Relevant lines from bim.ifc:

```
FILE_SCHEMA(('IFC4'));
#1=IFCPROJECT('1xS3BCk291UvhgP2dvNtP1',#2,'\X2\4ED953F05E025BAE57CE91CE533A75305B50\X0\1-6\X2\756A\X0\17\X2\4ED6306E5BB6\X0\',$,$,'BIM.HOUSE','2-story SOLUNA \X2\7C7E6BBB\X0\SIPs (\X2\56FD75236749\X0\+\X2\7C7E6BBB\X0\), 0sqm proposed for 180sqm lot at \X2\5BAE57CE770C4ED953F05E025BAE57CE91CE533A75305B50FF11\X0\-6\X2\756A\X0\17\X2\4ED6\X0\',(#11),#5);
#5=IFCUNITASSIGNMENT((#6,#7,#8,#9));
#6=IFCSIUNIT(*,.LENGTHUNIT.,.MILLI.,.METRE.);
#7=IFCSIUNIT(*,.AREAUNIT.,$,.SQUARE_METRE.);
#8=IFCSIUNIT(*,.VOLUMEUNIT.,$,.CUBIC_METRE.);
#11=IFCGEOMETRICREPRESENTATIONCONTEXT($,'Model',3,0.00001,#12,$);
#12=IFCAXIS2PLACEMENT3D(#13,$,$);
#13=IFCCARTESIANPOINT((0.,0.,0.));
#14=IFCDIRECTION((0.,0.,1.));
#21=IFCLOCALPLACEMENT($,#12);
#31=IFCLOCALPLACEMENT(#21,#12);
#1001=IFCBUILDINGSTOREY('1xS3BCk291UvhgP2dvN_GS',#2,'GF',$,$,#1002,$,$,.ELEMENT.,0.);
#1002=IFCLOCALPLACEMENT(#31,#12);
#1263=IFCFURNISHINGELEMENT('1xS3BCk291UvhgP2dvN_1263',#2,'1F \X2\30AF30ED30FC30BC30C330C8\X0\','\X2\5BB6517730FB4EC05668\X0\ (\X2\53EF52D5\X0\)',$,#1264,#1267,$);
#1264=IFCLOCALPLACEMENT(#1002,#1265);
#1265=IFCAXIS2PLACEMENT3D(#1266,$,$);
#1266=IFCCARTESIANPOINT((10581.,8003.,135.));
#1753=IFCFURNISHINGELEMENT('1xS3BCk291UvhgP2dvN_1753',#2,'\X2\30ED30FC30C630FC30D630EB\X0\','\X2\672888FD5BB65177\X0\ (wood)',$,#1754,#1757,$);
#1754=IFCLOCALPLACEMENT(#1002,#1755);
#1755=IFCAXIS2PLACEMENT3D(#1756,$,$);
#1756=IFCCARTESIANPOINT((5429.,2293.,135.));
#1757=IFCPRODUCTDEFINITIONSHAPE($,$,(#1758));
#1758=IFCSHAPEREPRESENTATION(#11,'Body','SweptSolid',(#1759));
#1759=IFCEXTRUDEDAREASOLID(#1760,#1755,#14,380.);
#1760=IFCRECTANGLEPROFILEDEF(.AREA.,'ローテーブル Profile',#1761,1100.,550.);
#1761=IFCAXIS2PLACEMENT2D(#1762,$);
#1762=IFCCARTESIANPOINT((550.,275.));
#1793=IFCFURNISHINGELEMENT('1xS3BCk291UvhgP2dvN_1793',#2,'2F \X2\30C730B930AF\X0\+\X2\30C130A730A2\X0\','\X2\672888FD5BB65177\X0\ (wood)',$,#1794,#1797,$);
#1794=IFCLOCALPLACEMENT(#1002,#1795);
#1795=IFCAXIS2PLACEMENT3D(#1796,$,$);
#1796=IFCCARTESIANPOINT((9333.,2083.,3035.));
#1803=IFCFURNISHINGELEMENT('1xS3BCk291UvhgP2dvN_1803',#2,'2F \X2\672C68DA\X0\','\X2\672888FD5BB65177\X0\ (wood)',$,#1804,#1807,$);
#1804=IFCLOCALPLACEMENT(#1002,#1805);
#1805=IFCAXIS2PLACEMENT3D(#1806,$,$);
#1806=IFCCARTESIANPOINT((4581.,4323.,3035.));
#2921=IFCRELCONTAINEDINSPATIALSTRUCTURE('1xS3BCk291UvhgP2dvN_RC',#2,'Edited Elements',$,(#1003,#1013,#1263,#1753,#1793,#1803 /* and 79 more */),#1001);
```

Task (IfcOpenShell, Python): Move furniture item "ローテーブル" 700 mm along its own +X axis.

```python
import ifcopenshell
import ifcopenshell.api.geometry
import ifcopenshell.util.placement
import ifcopenshell.util.unit

model = ifcopenshell.open("bim.ifc")
unit_scale = ifcopenshell.util.unit.calculate_unit_scale(model)

item = model.by_guid("1xS3BCk291UvhgP2dvN_1753")
matrix = ifcopenshell.util.placement.get_local_placement(item.ObjectPlacement)
matrix[:3, 3] += matrix[:3, 0] * 0.7 / unit_scale
ifcopenshell.api.geometry.edit_object_placement(model, product=item, matrix=matrix, is_si=False)

print(ifcopenshell.util.placement.get_local_placement(item.ObjectPlacement).round(3) + 0.0)

model.write("bim-out.ifc")
```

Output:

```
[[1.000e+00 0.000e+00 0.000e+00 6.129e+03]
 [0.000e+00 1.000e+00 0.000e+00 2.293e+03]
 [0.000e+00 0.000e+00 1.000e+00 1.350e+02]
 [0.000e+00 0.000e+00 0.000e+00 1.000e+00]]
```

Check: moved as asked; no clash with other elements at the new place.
